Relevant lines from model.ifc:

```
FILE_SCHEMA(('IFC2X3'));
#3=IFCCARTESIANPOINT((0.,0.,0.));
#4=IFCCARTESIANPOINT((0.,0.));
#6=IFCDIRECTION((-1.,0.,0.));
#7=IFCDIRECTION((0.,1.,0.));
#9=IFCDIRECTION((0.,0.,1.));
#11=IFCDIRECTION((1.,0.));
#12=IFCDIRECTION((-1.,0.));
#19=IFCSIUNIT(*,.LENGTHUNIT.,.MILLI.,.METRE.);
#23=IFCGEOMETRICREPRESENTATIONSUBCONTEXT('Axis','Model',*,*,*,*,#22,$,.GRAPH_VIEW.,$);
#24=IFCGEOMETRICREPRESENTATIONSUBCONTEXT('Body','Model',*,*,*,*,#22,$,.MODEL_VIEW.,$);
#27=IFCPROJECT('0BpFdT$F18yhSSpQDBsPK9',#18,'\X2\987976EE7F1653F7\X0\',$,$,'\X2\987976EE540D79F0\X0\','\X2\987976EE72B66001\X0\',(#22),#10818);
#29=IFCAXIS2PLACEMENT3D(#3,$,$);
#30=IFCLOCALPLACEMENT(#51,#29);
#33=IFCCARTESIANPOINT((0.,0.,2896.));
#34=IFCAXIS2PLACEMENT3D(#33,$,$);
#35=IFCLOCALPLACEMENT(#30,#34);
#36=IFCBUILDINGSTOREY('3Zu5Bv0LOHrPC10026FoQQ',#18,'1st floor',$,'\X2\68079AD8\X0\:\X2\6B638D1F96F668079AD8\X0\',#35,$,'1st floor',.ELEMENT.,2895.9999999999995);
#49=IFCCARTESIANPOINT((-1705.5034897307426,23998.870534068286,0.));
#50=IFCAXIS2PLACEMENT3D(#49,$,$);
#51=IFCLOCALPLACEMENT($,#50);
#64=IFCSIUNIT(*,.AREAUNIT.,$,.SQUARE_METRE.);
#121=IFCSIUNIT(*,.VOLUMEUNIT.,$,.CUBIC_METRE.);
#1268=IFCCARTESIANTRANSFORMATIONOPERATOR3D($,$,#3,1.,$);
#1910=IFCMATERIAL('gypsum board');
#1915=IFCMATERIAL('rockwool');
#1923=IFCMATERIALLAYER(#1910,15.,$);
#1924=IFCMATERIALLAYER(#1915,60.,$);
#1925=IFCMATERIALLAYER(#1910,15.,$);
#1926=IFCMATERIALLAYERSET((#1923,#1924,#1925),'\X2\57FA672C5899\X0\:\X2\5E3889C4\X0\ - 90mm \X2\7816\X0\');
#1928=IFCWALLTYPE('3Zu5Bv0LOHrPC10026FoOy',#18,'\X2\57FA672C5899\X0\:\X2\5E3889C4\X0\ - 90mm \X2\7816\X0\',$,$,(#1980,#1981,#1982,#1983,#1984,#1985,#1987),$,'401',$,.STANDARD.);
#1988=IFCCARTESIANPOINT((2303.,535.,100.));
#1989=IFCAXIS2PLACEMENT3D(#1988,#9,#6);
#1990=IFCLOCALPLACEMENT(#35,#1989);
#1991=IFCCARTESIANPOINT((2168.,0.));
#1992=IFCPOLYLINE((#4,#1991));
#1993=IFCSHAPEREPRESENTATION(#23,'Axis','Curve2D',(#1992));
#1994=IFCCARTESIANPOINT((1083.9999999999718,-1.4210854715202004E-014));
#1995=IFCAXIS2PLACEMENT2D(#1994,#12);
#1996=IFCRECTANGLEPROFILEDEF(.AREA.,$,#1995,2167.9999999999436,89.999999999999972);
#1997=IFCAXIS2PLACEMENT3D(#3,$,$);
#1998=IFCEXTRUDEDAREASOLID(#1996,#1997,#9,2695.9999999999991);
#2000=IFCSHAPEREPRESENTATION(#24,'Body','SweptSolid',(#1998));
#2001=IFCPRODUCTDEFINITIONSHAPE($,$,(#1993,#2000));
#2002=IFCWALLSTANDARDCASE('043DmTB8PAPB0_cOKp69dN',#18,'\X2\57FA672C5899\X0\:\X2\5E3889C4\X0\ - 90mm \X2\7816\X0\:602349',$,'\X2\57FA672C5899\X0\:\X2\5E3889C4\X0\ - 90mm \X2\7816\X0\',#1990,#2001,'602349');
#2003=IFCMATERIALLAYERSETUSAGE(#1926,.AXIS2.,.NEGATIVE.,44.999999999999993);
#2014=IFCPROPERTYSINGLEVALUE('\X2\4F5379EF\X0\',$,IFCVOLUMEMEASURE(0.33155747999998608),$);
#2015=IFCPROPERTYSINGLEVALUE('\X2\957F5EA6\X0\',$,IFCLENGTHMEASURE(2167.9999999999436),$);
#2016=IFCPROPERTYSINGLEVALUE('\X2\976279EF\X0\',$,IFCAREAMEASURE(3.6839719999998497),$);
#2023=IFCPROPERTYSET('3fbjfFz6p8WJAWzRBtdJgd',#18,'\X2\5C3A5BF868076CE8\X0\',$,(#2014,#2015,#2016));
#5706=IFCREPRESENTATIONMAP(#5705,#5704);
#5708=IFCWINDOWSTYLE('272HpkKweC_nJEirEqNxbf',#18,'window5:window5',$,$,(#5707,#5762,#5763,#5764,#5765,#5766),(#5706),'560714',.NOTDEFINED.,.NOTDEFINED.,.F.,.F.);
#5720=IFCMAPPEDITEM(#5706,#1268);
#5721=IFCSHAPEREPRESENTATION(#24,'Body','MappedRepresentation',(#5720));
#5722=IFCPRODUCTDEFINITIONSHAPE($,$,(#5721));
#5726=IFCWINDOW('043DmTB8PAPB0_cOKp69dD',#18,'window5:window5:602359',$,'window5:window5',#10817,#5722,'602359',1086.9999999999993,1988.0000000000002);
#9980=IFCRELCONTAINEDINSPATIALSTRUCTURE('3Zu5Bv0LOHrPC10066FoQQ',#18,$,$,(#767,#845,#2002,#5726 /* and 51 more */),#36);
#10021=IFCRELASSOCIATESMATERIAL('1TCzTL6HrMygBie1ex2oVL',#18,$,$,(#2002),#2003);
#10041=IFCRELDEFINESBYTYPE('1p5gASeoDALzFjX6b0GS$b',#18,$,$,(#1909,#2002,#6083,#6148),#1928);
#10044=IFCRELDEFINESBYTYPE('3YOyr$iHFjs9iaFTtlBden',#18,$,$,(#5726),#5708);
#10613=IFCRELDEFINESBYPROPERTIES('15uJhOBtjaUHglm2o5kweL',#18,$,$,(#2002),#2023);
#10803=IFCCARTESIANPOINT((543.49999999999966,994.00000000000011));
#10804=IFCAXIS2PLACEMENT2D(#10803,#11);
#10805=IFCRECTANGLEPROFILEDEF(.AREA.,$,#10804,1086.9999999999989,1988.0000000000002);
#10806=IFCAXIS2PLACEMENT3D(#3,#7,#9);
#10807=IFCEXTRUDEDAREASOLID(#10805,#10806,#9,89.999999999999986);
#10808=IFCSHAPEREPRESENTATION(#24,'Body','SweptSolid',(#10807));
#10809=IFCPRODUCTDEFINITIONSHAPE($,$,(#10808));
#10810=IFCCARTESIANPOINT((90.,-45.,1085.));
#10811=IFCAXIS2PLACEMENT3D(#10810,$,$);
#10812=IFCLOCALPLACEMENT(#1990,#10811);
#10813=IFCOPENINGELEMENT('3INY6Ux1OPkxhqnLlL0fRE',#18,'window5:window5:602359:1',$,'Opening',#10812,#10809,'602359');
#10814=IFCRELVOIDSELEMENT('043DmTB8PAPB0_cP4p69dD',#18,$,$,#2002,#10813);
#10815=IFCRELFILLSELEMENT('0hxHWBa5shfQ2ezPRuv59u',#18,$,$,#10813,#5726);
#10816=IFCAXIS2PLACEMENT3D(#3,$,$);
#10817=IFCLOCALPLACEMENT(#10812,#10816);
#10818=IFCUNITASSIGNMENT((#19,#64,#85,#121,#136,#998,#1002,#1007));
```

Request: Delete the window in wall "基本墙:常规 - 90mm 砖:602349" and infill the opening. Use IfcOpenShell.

```python
import ifcopenshell
import ifcopenshell.api.feature
import ifcopenshell.api.pset
import ifcopenshell.api.root
import ifcopenshell.geom
import ifcopenshell.util.element
import ifcopenshell.util.shape
import ifcopenshell.util.unit

model = ifcopenshell.open("model.ifc")
area_scale = ifcopenshell.util.unit.calculate_unit_scale(model, "AREAUNIT")
volume_scale = ifcopenshell.util.unit.calculate_unit_scale(model, "VOLUMEUNIT")
settings = ifcopenshell.geom.settings()


def volume(element):
    """Net volume in cubic metres, openings subtracted."""
    shape = ifcopenshell.geom.create_shape(settings, element)
    return ifcopenshell.util.shape.get_volume(shape.geometry)


window = model.by_id(5726)
opening = window.FillsVoids[0].RelatingOpeningElement
wall = opening.VoidsElements[0].RelatingBuildingElement
before = volume(wall)

ifcopenshell.api.root.remove_product(model, product=window)
ifcopenshell.api.feature.remove_feature(model, feature=opening)

after = volume(wall)
thickness = 0.09  # wall thickness in metres

# Update the wall's stored quantities.
pset = model.by_id(ifcopenshell.util.element.get_pset(wall, "尺寸标注", should_inherit=False)["id"])
ifcopenshell.api.pset.edit_pset(model, pset=pset, properties={
    "体积": model.create_entity("IfcVolumeMeasure", after / volume_scale),
    "面积": model.create_entity("IfcAreaMeasure", after / thickness / area_scale),
})

print(f"wall volume {before:.3f} -> {after:.3f} m3")

model.write("model_v2.ifc")
```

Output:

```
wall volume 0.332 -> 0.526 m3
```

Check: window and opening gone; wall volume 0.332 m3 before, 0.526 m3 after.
